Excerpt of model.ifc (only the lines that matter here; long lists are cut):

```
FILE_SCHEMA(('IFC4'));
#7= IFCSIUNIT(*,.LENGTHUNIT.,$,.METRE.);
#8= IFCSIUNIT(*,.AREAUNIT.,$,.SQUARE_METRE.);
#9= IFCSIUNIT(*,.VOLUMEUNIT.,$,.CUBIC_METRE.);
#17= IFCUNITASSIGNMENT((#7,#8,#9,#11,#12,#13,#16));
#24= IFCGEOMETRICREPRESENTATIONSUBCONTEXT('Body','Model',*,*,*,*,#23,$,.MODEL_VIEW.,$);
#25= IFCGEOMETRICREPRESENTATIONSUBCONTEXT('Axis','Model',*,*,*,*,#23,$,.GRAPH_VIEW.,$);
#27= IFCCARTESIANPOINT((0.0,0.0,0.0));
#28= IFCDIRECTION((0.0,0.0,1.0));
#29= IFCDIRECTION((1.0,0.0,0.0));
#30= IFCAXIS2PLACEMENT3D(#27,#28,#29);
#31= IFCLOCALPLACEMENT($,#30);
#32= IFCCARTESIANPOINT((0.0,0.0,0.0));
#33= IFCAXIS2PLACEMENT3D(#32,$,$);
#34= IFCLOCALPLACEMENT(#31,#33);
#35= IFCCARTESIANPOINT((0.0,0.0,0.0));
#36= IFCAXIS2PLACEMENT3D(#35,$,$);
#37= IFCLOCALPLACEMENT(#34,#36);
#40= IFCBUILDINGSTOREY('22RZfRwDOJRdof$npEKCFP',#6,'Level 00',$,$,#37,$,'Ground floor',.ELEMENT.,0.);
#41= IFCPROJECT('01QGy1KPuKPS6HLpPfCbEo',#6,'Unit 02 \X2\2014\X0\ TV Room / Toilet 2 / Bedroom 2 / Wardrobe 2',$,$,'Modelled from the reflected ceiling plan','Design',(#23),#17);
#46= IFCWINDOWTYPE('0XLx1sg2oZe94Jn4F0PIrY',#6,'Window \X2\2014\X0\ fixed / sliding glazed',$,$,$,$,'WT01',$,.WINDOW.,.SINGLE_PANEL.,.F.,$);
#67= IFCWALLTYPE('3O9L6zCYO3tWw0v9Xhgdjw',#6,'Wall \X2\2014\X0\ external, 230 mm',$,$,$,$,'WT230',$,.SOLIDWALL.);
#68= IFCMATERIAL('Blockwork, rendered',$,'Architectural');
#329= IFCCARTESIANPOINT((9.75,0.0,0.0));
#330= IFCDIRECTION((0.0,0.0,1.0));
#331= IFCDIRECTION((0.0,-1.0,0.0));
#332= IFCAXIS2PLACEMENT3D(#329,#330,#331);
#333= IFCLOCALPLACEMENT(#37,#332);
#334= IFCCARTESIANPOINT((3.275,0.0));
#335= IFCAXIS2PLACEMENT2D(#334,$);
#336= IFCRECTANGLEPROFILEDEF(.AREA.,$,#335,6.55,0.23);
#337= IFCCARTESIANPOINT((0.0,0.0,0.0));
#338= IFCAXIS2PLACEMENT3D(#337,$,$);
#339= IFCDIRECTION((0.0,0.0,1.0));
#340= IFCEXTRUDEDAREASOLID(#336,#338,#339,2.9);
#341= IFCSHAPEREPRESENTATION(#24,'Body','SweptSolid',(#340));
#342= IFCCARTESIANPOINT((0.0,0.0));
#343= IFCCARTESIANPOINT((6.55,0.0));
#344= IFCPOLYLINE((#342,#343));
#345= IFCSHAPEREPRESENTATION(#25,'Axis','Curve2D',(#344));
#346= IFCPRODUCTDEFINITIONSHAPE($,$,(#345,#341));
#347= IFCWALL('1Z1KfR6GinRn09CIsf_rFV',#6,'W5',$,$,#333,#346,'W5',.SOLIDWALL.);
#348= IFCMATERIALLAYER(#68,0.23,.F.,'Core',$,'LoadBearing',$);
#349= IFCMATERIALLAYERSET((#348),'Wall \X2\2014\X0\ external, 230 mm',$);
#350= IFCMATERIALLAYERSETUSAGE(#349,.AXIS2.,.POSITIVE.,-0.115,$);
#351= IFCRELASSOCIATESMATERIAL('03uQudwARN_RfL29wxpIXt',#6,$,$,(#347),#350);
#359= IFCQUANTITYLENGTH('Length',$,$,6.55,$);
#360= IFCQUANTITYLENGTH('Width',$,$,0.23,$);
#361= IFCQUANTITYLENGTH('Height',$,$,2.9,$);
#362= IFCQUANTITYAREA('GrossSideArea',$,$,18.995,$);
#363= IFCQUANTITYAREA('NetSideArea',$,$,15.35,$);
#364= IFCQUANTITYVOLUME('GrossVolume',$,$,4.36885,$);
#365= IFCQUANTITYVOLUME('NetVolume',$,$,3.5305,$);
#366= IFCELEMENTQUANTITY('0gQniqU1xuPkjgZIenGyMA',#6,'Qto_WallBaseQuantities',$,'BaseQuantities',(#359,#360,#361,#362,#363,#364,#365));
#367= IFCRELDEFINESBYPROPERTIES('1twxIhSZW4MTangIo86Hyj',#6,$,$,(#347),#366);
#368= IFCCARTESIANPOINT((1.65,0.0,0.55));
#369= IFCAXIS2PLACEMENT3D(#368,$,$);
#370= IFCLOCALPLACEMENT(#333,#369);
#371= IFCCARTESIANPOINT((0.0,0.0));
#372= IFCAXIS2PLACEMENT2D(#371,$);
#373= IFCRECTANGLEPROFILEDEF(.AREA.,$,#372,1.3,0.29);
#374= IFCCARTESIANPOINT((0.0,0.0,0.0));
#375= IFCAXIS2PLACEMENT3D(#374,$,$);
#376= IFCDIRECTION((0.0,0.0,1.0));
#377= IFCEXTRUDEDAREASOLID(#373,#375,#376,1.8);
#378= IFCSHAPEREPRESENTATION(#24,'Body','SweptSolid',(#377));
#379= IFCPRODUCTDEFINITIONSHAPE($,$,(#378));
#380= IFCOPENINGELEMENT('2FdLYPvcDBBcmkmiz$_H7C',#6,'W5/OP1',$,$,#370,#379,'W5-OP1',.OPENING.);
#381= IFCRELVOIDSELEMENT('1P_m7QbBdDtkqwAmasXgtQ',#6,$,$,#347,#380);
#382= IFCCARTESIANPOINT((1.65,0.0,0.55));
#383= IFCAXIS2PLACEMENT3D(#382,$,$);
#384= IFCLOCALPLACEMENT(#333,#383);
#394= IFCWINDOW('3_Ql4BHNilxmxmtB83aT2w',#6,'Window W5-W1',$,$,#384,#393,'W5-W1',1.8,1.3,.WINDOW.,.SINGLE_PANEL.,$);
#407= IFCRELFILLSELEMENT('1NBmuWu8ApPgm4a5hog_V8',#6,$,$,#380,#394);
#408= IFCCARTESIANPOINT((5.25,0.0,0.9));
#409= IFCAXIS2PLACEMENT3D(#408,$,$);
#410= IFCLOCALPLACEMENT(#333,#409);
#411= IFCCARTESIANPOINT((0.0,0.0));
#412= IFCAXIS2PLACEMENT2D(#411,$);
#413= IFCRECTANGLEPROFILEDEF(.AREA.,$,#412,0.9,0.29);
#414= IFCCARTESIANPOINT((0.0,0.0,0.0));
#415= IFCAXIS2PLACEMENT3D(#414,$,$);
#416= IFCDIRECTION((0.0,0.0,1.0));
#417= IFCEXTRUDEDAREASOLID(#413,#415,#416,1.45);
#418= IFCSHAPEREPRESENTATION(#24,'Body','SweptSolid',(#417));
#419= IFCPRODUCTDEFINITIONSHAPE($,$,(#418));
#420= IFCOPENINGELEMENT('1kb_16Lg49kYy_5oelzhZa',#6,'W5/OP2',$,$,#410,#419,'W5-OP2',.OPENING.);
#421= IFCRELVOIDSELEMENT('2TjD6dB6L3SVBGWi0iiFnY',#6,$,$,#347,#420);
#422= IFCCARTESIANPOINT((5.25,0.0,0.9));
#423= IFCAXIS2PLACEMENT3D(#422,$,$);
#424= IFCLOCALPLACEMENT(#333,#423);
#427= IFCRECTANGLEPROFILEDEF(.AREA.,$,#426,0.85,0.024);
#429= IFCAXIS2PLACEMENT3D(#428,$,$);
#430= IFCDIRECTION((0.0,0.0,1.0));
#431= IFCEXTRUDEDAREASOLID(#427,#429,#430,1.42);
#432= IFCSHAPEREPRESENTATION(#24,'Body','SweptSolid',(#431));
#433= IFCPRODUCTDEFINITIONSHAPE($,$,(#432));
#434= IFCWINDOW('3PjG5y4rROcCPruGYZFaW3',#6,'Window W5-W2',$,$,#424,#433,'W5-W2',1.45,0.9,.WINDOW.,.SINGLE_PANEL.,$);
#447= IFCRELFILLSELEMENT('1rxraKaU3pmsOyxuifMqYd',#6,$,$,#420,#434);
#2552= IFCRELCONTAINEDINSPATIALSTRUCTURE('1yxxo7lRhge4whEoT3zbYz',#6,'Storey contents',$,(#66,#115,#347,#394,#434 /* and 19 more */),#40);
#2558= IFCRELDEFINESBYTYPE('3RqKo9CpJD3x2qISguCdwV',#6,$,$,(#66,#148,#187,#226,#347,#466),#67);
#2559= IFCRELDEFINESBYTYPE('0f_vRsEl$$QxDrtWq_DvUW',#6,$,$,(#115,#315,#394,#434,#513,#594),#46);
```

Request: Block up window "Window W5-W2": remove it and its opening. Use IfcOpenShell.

```python
import ifcopenshell
import ifcopenshell.api.feature
import ifcopenshell.api.pset
import ifcopenshell.api.root
import ifcopenshell.geom
import ifcopenshell.util.element
import ifcopenshell.util.shape
import ifcopenshell.util.unit

model = ifcopenshell.open("model.ifc")
area_scale = ifcopenshell.util.unit.calculate_unit_scale(model, "AREAUNIT")
volume_scale = ifcopenshell.util.unit.calculate_unit_scale(model, "VOLUMEUNIT")
settings = ifcopenshell.geom.settings()


def volume(element):
    """Net volume in cubic metres, openings subtracted."""
    shape = ifcopenshell.geom.create_shape(settings, element)
    return ifcopenshell.util.shape.get_volume(shape.geometry)


window = model.by_id(434)
opening = window.FillsVoids[0].RelatingOpeningElement
wall = opening.VoidsElements[0].RelatingBuildingElement
before = volume(wall)

ifcopenshell.api.root.remove_product(model, product=window)
ifcopenshell.api.feature.remove_feature(model, feature=opening)

after = volume(wall)
thickness = 0.23  # wall thickness in metres

# Update the wall's stored quantities.
qto = model.by_id(ifcopenshell.util.element.get_pset(wall, "Qto_WallBaseQuantities", should_inherit=False)["id"])
ifcopenshell.api.pset.edit_qto(model, qto=qto, properties={
    "NetSideArea": after / thickness / area_scale,
    "NetVolume": after / volume_scale,
})

print(f"wall volume {before:.3f} -> {after:.3f} m3")

model.write("model_edited.ifc")
```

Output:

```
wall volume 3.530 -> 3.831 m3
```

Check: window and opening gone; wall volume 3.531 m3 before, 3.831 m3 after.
